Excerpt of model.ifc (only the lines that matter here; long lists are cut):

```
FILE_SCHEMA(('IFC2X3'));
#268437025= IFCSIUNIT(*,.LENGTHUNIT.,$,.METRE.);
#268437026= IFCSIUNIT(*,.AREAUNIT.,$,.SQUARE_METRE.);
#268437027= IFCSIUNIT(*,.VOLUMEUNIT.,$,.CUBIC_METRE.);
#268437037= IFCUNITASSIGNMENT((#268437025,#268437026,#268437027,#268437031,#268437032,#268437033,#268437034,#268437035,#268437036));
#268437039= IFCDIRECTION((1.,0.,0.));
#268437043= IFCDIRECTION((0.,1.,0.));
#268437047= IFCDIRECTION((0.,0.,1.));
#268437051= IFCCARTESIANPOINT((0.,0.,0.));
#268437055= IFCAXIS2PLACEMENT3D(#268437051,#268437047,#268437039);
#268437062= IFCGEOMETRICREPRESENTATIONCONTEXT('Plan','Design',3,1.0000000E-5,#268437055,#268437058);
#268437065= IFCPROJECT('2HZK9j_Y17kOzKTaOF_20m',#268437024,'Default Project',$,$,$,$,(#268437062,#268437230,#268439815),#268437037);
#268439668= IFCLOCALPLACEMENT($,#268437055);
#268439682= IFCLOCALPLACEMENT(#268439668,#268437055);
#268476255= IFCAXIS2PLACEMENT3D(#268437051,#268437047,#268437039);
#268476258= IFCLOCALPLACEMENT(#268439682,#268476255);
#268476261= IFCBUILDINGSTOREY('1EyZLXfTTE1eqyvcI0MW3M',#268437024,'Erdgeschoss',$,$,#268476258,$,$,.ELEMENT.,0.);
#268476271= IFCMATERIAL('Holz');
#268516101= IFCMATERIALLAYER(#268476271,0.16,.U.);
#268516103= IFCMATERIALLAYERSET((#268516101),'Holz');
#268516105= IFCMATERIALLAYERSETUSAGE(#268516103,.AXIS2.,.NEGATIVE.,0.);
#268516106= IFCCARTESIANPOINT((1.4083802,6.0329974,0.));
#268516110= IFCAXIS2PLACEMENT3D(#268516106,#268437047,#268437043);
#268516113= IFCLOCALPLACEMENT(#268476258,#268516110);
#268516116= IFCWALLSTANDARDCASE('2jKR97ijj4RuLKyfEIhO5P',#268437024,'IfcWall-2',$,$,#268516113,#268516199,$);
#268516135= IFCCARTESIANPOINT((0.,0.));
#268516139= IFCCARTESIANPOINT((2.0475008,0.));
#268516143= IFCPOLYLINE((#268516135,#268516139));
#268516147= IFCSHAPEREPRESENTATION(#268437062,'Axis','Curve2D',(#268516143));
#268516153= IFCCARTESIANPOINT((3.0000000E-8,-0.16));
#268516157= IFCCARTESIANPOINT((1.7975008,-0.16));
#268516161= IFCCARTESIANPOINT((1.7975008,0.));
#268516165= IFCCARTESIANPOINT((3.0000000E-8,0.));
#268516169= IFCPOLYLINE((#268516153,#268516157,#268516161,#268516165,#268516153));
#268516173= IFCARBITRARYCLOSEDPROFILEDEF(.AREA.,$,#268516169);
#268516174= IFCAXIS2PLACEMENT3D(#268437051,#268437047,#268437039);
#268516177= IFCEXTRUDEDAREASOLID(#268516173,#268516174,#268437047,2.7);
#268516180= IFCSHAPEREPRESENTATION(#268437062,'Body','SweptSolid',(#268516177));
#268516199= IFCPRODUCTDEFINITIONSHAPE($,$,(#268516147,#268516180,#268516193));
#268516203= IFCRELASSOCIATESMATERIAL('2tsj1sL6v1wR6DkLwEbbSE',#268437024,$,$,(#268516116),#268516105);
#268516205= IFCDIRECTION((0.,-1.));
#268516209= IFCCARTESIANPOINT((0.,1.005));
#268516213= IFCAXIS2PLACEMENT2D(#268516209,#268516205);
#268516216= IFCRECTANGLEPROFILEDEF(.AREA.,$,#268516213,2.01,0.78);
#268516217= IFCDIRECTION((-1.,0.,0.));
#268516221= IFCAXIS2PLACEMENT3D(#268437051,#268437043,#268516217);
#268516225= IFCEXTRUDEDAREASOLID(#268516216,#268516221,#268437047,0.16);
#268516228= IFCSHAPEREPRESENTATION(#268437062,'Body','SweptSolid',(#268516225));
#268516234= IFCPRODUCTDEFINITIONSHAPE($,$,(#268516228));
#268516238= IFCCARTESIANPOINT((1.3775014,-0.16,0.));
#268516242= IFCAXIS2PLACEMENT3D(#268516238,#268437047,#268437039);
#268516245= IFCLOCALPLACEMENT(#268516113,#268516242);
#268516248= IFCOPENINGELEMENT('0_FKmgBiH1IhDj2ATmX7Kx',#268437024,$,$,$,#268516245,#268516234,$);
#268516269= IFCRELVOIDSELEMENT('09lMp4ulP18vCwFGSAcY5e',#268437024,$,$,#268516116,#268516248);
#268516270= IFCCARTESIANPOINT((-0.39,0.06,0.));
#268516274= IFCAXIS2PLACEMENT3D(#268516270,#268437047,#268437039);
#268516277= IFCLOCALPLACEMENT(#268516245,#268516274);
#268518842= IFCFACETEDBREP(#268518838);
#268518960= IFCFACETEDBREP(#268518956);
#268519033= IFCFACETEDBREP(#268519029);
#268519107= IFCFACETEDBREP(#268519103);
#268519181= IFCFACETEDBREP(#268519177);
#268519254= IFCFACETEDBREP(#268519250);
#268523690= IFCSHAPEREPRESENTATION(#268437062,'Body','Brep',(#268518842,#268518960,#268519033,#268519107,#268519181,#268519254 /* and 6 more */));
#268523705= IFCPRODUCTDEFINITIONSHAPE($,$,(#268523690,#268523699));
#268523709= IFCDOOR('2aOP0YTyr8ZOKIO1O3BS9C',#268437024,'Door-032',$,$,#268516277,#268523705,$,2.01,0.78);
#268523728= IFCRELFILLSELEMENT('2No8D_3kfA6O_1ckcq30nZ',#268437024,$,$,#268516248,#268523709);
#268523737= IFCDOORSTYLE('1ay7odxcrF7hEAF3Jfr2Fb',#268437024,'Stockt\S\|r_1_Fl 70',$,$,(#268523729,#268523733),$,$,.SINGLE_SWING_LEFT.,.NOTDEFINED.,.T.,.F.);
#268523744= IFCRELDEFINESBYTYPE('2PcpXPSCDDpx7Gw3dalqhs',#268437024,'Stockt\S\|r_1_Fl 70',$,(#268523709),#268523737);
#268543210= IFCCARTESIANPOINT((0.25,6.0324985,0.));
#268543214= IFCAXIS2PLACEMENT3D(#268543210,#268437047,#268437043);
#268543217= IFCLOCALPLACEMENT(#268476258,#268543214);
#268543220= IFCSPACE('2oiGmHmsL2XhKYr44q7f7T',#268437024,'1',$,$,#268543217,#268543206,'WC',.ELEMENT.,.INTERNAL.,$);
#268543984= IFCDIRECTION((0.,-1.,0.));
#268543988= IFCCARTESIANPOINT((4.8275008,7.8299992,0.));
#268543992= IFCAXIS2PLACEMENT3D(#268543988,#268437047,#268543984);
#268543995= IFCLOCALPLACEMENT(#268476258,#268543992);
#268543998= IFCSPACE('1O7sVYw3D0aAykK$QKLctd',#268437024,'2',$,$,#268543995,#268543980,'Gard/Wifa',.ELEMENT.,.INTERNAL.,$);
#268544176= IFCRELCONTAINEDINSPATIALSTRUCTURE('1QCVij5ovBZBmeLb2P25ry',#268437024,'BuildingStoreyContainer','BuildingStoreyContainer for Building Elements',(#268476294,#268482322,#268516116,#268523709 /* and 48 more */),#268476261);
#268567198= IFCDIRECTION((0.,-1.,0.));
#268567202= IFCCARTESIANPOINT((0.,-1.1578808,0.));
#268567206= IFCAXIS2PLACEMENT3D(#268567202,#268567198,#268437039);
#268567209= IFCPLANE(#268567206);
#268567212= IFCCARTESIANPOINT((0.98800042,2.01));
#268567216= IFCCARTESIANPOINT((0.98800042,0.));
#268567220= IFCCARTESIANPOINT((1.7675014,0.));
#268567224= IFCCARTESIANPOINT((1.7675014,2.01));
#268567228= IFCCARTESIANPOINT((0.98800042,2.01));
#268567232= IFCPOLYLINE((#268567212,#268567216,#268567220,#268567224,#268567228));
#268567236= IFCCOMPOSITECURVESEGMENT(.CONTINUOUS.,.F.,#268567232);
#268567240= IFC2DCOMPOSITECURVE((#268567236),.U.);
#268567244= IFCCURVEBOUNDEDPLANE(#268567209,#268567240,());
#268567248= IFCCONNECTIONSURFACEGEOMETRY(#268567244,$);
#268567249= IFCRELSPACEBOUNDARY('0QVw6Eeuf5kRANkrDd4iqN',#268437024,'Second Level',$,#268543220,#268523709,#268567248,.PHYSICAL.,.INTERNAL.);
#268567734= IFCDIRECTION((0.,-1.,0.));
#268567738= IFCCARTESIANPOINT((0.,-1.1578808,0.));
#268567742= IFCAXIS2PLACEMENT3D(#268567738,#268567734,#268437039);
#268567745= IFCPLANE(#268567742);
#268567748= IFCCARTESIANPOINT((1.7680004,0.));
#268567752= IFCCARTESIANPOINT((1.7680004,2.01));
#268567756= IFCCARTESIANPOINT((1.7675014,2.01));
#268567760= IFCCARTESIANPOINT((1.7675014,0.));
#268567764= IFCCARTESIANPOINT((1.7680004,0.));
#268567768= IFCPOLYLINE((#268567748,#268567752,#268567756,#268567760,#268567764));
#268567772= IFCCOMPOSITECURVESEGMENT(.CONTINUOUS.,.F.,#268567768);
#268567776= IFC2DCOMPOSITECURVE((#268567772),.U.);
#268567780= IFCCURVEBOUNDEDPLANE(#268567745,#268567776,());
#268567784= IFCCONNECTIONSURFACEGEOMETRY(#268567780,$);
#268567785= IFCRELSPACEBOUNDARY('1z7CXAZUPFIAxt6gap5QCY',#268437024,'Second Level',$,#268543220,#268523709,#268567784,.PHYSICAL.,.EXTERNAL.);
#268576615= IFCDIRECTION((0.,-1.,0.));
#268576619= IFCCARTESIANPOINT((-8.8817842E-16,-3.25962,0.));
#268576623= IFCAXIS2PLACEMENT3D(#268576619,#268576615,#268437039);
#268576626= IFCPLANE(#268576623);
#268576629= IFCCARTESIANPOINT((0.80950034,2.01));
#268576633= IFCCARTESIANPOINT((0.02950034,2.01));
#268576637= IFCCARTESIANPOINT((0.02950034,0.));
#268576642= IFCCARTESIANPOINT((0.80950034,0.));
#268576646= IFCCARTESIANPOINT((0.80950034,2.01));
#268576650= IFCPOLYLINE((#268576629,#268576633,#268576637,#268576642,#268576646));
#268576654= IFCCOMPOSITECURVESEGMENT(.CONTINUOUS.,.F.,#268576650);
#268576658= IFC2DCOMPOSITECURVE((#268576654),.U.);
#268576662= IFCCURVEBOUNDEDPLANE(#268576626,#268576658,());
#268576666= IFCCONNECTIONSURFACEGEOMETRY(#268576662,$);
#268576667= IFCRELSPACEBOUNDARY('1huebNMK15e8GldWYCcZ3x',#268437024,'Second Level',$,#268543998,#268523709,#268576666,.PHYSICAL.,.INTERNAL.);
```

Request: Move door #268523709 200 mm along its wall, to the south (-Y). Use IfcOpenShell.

```python
import numpy as np
import ifcopenshell
import ifcopenshell.api.geometry
import ifcopenshell.util.placement
import ifcopenshell.util.unit

model = ifcopenshell.open("model.ifc")
unit_scale = ifcopenshell.util.unit.calculate_unit_scale(model)

door = model.by_guid("2aOP0YTyr8ZOKIO1O3BS9C")
opening = door.FillsVoids[0].RelatingOpeningElement
wall = opening.VoidsElements[0].RelatingBuildingElement

wall_matrix = ifcopenshell.util.placement.get_local_placement(wall.ObjectPlacement)
shift = wall_matrix[:3, 0] * -0.2 / unit_scale
before = ifcopenshell.util.placement.get_local_placement(door.ObjectPlacement)[:3, 3].copy()

# The door is placed relative to its opening, so it follows when the opening moves.
matrix = ifcopenshell.util.placement.get_local_placement(opening.ObjectPlacement)
matrix[:3, 3] += shift
ifcopenshell.api.geometry.edit_object_placement(
    model, product=opening, matrix=matrix, is_si=False, should_transform_children=True
)

# Space boundary surfaces are stored in each space's coordinates; move them too.
for rel in door.ProvidesBoundaries:
    if not rel.ConnectionGeometry:
        continue
    surface = rel.ConnectionGeometry.SurfaceOnRelatingElement.BasisSurface
    space_matrix = ifcopenshell.util.placement.get_local_placement(rel.RelatingSpace.ObjectPlacement)
    point = np.array(surface.Position.Location.Coordinates) + space_matrix[:3, :3].T @ shift
    surface.Position = model.createIfcAxis2Placement3D(
        model.createIfcCartesianPoint(point.tolist()), surface.Position.Axis, surface.Position.RefDirection
    )

after = ifcopenshell.util.placement.get_local_placement(door.ObjectPlacement)[:3, 3]
print("door moved by", (after - before).round(3) + 0.0)

model.write("model_rev.ifc")
```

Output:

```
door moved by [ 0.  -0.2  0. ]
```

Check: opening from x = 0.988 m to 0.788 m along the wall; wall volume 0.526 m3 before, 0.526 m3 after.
